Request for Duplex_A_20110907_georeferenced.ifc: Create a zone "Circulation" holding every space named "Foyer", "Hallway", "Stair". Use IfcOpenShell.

First a look at what the model holds.

```python
import ifcopenshell

model = ifcopenshell.open("Duplex_A_20110907_georeferenced.ifc")
print(model.schema)
seen = {}
for space in model.by_type("IfcSpace"):
    seen[space.LongName] = seen.get(space.LongName, 0) + 1
for name, count in sorted(seen.items(), key=str):
    print(count, "x", name)
print("zones:", [z.Name for z in model.by_type("IfcZone")][:20])
```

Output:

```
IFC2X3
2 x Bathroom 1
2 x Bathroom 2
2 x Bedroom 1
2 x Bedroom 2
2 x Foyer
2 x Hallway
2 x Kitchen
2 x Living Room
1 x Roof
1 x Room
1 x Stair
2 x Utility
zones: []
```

```python
import ifcopenshell
import ifcopenshell.api.group
import ifcopenshell.api.root

model = ifcopenshell.open("Duplex_A_20110907_georeferenced.ifc")

names = {"Foyer", "Hallway", "Stair"}
spaces = [s for s in model.by_type("IfcSpace") if s.LongName in names]

zone = ifcopenshell.api.root.create_entity(model, ifc_class="IfcZone", name="Circulation")
ifcopenshell.api.group.assign_group(model, products=spaces, group=zone)
print(len(spaces), "spaces in", zone.Name)

model.write("Duplex_A_20110907_georeferenced-out.ifc")
```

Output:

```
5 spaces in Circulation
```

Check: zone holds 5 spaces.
